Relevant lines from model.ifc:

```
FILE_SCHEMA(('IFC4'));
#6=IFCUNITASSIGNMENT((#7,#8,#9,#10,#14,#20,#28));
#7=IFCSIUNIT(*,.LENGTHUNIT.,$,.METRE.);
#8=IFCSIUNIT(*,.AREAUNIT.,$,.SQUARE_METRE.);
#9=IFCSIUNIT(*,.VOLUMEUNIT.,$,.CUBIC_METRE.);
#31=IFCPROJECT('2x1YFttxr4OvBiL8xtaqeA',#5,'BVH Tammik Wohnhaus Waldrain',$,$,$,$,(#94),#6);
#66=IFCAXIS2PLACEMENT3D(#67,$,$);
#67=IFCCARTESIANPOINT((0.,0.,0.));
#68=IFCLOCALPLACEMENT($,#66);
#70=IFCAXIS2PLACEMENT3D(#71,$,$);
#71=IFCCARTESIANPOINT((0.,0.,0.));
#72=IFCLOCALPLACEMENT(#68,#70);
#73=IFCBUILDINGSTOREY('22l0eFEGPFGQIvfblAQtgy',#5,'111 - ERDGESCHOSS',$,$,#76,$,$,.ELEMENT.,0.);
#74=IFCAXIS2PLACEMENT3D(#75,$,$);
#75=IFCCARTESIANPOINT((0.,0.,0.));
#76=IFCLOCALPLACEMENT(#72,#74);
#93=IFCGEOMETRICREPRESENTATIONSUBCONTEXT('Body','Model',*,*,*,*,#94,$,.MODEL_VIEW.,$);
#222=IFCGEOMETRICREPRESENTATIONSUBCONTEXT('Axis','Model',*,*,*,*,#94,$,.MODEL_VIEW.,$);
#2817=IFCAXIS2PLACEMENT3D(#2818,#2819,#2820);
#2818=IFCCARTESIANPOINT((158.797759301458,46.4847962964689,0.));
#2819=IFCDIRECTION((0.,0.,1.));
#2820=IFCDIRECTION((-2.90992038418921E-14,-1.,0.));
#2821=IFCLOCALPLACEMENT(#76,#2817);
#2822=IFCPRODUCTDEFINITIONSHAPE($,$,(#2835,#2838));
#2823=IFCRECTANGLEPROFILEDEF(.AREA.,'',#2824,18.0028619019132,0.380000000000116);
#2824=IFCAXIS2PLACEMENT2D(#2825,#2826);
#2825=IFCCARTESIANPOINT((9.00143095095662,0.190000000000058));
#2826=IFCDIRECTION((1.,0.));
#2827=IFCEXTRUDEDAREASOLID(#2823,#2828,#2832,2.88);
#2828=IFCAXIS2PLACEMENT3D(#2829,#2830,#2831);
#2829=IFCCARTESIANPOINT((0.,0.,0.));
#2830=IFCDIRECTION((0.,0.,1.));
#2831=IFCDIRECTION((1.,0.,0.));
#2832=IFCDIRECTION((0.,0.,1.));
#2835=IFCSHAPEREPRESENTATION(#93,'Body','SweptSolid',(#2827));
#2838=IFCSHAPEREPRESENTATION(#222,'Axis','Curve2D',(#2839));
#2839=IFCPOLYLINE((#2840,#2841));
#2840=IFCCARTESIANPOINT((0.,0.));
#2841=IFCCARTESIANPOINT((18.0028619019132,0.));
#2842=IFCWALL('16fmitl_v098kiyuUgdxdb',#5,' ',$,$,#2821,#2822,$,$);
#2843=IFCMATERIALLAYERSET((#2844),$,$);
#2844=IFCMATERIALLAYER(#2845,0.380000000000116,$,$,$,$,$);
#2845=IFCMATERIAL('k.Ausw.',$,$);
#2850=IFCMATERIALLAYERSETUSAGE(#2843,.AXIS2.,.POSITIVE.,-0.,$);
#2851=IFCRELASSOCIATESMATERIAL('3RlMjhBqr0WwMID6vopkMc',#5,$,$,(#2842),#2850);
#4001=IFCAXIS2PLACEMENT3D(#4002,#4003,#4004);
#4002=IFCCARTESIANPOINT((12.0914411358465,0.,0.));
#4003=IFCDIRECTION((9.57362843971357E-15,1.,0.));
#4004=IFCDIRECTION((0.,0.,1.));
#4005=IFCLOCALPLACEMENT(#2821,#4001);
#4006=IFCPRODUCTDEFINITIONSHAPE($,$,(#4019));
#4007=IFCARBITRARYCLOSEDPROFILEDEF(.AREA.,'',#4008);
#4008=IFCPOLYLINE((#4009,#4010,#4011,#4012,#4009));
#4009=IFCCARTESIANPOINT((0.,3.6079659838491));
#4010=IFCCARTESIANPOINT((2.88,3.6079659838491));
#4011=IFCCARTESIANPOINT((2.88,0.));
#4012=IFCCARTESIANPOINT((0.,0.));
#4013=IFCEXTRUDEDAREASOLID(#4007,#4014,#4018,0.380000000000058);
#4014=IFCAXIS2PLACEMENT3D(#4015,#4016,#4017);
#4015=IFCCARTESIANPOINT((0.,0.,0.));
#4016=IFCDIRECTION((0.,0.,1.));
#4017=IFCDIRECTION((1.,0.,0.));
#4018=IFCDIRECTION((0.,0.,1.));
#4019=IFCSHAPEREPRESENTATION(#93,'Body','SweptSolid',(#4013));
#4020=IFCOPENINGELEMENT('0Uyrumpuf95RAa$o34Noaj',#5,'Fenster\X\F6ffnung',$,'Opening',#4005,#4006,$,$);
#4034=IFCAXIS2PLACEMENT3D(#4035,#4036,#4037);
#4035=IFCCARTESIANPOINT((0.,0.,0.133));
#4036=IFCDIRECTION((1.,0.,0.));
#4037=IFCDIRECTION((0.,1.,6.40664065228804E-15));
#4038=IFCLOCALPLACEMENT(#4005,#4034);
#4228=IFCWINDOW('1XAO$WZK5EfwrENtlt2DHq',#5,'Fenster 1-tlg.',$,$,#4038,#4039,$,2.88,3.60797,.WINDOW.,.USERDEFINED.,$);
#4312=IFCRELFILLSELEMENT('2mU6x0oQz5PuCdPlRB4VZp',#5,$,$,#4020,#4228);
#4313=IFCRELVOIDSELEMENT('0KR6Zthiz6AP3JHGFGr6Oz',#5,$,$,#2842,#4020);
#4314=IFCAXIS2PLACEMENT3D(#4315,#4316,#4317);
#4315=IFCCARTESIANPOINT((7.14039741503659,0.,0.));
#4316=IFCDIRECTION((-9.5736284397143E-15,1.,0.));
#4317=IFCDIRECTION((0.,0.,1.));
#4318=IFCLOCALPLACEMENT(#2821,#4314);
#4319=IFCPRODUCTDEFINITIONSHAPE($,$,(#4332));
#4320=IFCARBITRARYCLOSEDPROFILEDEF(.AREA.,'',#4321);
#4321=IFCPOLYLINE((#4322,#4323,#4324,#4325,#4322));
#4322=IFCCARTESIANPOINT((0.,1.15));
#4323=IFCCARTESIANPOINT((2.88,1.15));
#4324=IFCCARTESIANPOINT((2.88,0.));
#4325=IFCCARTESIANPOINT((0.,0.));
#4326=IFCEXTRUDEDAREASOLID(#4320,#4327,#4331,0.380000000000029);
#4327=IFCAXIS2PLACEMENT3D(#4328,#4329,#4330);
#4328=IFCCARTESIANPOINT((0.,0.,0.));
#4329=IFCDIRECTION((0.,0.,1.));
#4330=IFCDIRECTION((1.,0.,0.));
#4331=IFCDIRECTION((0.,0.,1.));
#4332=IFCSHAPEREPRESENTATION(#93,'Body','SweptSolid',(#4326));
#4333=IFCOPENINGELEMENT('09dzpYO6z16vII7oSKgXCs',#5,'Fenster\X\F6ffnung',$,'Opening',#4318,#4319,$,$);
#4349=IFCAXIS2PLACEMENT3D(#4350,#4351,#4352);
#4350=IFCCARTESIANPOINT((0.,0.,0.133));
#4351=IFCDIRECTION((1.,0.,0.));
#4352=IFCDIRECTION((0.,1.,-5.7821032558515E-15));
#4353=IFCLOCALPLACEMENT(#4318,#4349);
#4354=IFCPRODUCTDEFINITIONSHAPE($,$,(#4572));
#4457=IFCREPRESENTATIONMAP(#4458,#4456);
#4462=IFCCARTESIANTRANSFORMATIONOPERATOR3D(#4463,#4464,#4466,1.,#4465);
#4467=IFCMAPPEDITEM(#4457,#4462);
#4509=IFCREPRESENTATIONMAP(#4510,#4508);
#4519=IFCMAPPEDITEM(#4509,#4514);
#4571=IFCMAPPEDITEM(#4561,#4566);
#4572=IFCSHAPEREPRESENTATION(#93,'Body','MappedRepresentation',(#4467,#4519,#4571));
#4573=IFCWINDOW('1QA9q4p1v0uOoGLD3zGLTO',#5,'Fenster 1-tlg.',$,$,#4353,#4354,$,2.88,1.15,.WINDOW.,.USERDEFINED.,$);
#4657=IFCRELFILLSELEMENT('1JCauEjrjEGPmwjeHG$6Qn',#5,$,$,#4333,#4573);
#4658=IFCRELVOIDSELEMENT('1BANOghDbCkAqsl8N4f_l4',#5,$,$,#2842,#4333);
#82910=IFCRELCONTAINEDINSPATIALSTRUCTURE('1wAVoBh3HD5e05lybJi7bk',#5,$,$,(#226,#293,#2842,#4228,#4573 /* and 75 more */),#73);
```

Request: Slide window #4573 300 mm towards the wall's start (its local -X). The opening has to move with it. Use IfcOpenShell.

```python
import ifcopenshell
import ifcopenshell.api.geometry
import ifcopenshell.util.placement
import ifcopenshell.util.unit

model = ifcopenshell.open("model.ifc")
unit_scale = ifcopenshell.util.unit.calculate_unit_scale(model)

window = model.by_guid("1QA9q4p1v0uOoGLD3zGLTO")
opening = window.FillsVoids[0].RelatingOpeningElement
wall = opening.VoidsElements[0].RelatingBuildingElement

wall_matrix = ifcopenshell.util.placement.get_local_placement(wall.ObjectPlacement)
shift = wall_matrix[:3, 0] * -0.3 / unit_scale
before = ifcopenshell.util.placement.get_local_placement(window.ObjectPlacement)[:3, 3].copy()

# The window is placed relative to its opening, so it follows when the opening moves.
matrix = ifcopenshell.util.placement.get_local_placement(opening.ObjectPlacement)
matrix[:3, 3] += shift
ifcopenshell.api.geometry.edit_object_placement(
    model, product=opening, matrix=matrix, is_si=False, should_transform_children=True
)

after = ifcopenshell.util.placement.get_local_placement(window.ObjectPlacement)[:3, 3]
print("window moved by", (after - before).round(3) + 0.0)

model.write("model-out.ifc")
```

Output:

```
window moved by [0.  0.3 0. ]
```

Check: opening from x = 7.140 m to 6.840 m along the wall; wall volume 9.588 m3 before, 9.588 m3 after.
